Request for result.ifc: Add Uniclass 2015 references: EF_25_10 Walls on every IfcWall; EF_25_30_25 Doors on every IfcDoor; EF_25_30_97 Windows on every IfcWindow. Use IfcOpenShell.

First a look at what the model holds.

```python
import ifcopenshell

model = ifcopenshell.open("result.ifc")
print(model.schema)
print("classifications:", [c.Name for c in model.by_type("IfcClassification")])
for ifc_class in ("IfcDoor", "IfcRoof", "IfcStair", "IfcWall", "IfcWindow"):
    print(ifc_class, len(model.by_type(ifc_class)))
```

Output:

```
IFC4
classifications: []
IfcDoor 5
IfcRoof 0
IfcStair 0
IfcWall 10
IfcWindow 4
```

```python
import ifcopenshell
import ifcopenshell.api.classification

model = ifcopenshell.open("result.ifc")

system = ifcopenshell.api.classification.add_classification(model, classification="Uniclass 2015")

codes = {
    "IfcWall": ("EF_25_10", "Walls"),
    "IfcDoor": ("EF_25_30_25", "Doors"),
    "IfcWindow": ("EF_25_30_97", "Windows"),
}
for ifc_class, (code, name) in codes.items():
    products = model.by_type(ifc_class)
    ifcopenshell.api.classification.add_reference(
        model, products=products, classification=system, identification=code, name=name
    )
    print(code, len(products))

model.write("result_v2.ifc")
```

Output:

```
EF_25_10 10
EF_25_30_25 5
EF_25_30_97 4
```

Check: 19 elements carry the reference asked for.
